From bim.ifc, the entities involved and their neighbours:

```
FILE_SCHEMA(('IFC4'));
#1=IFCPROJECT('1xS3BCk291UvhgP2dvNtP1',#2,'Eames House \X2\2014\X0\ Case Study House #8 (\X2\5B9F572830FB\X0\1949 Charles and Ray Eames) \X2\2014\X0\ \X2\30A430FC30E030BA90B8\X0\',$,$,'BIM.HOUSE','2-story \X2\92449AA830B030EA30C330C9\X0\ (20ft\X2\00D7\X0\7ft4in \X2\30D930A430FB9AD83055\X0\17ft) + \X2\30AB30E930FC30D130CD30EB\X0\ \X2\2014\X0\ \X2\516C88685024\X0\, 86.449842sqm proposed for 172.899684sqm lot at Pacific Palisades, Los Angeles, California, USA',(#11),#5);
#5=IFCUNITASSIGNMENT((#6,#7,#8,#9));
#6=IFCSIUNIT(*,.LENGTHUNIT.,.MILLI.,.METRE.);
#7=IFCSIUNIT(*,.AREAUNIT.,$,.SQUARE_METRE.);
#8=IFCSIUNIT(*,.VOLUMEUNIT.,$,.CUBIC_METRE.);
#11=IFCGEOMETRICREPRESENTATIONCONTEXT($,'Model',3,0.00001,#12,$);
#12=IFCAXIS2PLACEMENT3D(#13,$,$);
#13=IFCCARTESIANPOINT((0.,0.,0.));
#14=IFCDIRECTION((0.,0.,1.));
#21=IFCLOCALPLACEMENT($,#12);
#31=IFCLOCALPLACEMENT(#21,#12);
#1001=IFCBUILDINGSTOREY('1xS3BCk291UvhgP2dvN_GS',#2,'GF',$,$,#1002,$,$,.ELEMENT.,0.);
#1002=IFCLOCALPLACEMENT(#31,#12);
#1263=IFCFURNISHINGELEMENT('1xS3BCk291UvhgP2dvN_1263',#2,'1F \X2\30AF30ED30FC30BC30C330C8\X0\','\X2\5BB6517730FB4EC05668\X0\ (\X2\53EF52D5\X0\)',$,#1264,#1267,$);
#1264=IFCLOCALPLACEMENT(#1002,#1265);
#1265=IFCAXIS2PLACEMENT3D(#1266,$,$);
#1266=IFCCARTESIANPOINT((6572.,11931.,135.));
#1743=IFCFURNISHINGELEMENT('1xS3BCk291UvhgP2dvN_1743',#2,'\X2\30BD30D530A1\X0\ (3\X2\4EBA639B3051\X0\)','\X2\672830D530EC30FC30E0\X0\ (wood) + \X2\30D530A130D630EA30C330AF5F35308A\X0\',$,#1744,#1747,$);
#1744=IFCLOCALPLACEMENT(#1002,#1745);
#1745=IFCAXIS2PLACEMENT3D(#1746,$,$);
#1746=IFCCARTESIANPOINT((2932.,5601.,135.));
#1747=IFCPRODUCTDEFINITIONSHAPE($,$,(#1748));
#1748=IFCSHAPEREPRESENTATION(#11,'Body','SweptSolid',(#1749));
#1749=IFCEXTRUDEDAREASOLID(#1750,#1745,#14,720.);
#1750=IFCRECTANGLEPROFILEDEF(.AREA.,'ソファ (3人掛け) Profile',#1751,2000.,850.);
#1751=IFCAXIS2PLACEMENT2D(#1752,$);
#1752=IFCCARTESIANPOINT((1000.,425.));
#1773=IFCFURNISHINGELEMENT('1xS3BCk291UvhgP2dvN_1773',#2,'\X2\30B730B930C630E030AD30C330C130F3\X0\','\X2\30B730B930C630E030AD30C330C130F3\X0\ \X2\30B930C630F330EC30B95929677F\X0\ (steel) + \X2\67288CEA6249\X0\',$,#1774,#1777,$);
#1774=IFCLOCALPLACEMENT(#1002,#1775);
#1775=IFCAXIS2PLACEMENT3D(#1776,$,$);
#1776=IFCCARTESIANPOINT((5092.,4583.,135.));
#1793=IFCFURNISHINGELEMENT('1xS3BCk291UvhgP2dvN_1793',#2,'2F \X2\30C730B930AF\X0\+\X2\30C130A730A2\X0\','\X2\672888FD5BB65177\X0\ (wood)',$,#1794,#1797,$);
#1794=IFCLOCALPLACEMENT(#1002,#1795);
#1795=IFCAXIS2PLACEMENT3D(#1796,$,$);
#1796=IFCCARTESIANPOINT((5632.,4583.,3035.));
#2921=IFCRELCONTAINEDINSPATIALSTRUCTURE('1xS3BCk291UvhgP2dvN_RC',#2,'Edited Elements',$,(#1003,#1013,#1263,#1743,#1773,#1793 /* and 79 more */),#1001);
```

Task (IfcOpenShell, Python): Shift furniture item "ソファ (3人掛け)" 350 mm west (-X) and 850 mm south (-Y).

```python
import ifcopenshell
import ifcopenshell.api.geometry
import ifcopenshell.util.placement

model = ifcopenshell.open("bim.ifc")

item = model.by_guid("1xS3BCk291UvhgP2dvN_1743")
matrix = ifcopenshell.util.placement.get_local_placement(item.ObjectPlacement)
matrix[0, 3] -= 350.0
matrix[1, 3] -= 850.0
ifcopenshell.api.geometry.edit_object_placement(model, product=item, matrix=matrix, is_si=False)

print(ifcopenshell.util.placement.get_local_placement(item.ObjectPlacement).round(3) + 0.0)

model.write("bim_updated.ifc")
```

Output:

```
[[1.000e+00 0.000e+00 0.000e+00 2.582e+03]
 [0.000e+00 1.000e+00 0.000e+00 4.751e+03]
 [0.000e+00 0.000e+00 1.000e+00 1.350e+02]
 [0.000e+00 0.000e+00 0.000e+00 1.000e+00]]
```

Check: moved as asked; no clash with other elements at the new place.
